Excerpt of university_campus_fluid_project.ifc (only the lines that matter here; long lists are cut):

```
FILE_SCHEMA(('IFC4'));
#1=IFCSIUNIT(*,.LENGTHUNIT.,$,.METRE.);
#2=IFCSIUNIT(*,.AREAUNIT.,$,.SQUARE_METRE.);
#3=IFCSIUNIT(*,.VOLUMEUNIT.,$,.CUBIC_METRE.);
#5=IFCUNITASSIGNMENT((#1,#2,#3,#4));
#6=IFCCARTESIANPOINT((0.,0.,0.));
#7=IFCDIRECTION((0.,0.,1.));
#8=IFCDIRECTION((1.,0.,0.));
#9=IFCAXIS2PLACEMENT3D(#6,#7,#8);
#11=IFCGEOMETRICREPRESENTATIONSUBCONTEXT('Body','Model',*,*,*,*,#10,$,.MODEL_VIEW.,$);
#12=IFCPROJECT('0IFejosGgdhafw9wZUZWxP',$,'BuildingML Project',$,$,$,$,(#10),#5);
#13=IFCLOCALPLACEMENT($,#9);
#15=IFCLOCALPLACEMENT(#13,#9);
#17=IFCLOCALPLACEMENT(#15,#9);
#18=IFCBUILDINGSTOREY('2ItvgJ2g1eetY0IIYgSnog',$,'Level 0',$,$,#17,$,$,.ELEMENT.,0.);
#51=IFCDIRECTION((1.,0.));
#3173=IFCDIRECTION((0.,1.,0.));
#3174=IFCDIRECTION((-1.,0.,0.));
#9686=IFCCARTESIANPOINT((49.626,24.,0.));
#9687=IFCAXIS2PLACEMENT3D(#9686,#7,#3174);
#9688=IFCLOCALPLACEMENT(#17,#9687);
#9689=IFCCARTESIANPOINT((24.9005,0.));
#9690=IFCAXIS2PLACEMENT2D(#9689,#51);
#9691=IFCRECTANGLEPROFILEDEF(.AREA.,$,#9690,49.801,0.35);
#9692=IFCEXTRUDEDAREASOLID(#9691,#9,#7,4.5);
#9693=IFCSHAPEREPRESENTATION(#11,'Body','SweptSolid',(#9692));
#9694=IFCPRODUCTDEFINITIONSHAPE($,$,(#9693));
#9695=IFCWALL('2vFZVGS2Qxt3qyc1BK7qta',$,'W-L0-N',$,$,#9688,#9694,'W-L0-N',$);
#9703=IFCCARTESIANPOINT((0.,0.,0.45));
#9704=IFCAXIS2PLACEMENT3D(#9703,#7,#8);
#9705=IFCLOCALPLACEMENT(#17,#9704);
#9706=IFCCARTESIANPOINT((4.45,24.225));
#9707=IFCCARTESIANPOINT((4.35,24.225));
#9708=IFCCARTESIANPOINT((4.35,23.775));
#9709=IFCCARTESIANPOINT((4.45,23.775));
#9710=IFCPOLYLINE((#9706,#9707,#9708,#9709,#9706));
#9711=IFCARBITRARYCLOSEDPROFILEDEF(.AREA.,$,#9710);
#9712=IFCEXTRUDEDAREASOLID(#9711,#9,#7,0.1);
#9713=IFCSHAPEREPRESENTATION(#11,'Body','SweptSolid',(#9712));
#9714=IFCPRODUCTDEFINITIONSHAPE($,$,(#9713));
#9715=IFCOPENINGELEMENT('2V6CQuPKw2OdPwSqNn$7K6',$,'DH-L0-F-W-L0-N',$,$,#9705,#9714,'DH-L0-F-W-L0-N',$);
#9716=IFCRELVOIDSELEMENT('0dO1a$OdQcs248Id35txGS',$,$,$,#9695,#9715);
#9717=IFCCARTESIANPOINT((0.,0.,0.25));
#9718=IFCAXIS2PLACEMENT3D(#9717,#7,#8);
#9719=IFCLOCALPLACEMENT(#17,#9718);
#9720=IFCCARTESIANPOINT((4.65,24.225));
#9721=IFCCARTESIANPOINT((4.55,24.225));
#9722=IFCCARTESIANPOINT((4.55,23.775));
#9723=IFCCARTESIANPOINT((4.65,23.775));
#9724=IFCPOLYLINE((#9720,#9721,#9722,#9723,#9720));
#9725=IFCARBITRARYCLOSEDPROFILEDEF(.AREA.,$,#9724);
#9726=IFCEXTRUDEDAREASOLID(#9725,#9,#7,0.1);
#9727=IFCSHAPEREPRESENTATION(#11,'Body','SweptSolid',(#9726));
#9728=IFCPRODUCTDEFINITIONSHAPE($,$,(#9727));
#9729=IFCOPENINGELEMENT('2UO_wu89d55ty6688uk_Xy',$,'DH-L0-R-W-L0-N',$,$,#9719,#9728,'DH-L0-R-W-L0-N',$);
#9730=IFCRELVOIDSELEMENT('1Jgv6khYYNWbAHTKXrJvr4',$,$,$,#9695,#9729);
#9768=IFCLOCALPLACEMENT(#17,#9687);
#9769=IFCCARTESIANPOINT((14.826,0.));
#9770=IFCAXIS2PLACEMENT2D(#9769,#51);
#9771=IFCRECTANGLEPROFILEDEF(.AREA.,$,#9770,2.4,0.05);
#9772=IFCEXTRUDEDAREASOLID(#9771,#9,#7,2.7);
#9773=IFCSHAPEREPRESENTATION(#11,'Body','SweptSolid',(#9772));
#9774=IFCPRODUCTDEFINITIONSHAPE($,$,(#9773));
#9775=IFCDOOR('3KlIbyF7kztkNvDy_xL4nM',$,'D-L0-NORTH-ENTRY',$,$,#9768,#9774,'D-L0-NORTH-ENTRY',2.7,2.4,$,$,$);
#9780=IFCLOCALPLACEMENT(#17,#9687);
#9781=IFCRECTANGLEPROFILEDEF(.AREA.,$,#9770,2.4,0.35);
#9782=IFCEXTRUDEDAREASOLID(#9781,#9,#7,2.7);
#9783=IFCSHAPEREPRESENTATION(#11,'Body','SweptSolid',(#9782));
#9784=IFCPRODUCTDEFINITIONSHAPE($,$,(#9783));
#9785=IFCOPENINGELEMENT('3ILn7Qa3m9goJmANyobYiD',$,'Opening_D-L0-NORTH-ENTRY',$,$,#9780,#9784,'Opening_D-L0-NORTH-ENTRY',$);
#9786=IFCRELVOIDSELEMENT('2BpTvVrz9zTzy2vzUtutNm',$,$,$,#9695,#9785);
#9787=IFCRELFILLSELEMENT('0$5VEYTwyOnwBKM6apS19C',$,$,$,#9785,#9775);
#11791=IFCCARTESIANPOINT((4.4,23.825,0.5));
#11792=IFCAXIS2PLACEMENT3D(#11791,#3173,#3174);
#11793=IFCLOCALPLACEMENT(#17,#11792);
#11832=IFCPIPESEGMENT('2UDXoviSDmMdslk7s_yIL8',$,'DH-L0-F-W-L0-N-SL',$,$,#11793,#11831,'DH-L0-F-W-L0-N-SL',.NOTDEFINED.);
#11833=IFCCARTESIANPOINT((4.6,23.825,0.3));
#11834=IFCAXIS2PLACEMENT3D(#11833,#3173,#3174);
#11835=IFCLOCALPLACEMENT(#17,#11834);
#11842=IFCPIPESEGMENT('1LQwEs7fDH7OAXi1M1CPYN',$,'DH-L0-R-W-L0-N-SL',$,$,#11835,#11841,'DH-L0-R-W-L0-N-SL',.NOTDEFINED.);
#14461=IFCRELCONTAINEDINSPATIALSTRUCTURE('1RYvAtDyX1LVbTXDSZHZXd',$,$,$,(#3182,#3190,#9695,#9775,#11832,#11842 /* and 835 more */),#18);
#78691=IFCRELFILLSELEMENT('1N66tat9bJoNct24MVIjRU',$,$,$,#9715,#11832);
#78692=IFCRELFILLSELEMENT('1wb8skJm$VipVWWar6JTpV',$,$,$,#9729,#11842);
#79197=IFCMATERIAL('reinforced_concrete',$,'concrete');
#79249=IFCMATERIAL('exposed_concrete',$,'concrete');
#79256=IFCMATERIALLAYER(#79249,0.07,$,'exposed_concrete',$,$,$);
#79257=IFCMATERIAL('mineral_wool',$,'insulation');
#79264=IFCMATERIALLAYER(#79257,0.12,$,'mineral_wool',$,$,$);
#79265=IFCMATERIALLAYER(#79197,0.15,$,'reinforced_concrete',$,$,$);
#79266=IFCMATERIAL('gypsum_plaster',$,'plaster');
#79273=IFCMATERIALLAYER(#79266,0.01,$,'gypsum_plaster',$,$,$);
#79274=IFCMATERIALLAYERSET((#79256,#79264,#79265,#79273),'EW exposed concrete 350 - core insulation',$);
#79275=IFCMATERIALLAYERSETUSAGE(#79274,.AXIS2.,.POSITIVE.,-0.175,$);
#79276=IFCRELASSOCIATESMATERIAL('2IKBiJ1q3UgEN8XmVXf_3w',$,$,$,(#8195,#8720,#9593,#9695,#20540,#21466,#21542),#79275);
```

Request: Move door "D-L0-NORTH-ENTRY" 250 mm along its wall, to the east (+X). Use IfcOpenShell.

```python
import ifcopenshell
import ifcopenshell.api.geometry
import ifcopenshell.util.placement
import ifcopenshell.util.unit

model = ifcopenshell.open("university_campus_fluid_project.ifc")
unit_scale = ifcopenshell.util.unit.calculate_unit_scale(model)

door = model.by_guid("3KlIbyF7kztkNvDy_xL4nM")
opening = door.FillsVoids[0].RelatingOpeningElement
wall = opening.VoidsElements[0].RelatingBuildingElement

wall_matrix = ifcopenshell.util.placement.get_local_placement(wall.ObjectPlacement)
shift = wall_matrix[:3, 0] * -0.25 / unit_scale
before = ifcopenshell.util.placement.get_local_placement(door.ObjectPlacement)[:3, 3].copy()

# The door is not placed relative to its opening, so move both.
for product in (opening, door):
    matrix = ifcopenshell.util.placement.get_local_placement(product.ObjectPlacement)
    matrix[:3, 3] += shift
    ifcopenshell.api.geometry.edit_object_placement(model, product=product, matrix=matrix, is_si=False)

after = ifcopenshell.util.placement.get_local_placement(door.ObjectPlacement)[:3, 3]
print("door moved by", (after - before).round(3) + 0.0)

model.write("university_campus_fluid_project_v2.ifc")
```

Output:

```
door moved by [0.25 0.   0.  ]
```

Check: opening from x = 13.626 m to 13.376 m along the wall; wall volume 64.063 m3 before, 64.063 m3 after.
